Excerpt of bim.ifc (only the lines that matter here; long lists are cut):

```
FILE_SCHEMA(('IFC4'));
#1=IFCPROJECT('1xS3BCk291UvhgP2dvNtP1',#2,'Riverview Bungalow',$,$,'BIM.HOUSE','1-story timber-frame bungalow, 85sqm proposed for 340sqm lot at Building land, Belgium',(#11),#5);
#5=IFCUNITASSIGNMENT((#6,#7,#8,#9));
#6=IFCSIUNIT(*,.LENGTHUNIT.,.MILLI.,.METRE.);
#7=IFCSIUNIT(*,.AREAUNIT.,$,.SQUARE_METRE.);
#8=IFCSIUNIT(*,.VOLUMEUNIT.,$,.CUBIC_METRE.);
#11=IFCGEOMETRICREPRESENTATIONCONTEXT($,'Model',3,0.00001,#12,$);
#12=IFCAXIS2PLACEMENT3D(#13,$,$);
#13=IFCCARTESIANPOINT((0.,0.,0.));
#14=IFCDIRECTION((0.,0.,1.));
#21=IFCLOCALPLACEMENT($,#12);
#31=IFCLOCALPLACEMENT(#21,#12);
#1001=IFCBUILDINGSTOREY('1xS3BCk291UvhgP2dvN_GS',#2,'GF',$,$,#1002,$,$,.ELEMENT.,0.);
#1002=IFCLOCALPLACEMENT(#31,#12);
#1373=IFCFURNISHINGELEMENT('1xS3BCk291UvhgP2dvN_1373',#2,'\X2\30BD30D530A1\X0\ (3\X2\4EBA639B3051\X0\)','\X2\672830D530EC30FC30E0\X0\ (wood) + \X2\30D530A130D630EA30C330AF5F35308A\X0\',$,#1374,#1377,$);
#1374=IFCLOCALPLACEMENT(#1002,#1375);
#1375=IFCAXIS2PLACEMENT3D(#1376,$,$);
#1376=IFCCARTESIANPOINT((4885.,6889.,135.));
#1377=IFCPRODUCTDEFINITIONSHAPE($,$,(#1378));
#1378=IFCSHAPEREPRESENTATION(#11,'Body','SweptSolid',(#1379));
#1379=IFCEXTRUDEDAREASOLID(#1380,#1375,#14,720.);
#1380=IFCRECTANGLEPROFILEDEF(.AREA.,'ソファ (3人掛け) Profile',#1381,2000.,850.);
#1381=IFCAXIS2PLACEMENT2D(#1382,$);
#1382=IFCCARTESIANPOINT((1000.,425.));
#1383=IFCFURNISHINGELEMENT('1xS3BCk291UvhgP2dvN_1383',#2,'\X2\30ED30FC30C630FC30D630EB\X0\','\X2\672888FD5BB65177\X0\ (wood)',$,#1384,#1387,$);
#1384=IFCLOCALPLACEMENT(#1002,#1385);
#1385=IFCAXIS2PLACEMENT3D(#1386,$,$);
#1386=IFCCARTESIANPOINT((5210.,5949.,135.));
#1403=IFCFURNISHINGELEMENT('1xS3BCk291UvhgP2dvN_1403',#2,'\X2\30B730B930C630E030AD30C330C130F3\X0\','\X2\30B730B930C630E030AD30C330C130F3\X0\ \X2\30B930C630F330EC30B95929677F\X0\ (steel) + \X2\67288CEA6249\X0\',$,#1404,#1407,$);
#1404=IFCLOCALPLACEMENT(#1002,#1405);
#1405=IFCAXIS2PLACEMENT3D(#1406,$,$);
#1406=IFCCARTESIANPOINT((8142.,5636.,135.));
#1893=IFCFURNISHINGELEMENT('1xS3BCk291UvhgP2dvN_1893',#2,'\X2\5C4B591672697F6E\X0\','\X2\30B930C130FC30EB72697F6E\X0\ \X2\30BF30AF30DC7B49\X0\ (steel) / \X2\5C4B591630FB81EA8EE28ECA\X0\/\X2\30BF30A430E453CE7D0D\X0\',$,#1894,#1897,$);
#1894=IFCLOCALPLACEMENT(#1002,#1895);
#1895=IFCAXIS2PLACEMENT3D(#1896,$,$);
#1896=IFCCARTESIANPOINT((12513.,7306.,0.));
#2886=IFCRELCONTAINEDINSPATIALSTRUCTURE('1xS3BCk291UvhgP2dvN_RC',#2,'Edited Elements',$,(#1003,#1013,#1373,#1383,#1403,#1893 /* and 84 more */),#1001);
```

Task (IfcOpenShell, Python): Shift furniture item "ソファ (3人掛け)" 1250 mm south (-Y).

```python
import ifcopenshell
import ifcopenshell.api.geometry
import ifcopenshell.util.placement

model = ifcopenshell.open("bim.ifc")

item = model.by_guid("1xS3BCk291UvhgP2dvN_1373")
matrix = ifcopenshell.util.placement.get_local_placement(item.ObjectPlacement)
matrix[1, 3] -= 1250.0
ifcopenshell.api.geometry.edit_object_placement(model, product=item, matrix=matrix, is_si=False)

print(ifcopenshell.util.placement.get_local_placement(item.ObjectPlacement).round(3) + 0.0)

model.write("bim-out.ifc")
```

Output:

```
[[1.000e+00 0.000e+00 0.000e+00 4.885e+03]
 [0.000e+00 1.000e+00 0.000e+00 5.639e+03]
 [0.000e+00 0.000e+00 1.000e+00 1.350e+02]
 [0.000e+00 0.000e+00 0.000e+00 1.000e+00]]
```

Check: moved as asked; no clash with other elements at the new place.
